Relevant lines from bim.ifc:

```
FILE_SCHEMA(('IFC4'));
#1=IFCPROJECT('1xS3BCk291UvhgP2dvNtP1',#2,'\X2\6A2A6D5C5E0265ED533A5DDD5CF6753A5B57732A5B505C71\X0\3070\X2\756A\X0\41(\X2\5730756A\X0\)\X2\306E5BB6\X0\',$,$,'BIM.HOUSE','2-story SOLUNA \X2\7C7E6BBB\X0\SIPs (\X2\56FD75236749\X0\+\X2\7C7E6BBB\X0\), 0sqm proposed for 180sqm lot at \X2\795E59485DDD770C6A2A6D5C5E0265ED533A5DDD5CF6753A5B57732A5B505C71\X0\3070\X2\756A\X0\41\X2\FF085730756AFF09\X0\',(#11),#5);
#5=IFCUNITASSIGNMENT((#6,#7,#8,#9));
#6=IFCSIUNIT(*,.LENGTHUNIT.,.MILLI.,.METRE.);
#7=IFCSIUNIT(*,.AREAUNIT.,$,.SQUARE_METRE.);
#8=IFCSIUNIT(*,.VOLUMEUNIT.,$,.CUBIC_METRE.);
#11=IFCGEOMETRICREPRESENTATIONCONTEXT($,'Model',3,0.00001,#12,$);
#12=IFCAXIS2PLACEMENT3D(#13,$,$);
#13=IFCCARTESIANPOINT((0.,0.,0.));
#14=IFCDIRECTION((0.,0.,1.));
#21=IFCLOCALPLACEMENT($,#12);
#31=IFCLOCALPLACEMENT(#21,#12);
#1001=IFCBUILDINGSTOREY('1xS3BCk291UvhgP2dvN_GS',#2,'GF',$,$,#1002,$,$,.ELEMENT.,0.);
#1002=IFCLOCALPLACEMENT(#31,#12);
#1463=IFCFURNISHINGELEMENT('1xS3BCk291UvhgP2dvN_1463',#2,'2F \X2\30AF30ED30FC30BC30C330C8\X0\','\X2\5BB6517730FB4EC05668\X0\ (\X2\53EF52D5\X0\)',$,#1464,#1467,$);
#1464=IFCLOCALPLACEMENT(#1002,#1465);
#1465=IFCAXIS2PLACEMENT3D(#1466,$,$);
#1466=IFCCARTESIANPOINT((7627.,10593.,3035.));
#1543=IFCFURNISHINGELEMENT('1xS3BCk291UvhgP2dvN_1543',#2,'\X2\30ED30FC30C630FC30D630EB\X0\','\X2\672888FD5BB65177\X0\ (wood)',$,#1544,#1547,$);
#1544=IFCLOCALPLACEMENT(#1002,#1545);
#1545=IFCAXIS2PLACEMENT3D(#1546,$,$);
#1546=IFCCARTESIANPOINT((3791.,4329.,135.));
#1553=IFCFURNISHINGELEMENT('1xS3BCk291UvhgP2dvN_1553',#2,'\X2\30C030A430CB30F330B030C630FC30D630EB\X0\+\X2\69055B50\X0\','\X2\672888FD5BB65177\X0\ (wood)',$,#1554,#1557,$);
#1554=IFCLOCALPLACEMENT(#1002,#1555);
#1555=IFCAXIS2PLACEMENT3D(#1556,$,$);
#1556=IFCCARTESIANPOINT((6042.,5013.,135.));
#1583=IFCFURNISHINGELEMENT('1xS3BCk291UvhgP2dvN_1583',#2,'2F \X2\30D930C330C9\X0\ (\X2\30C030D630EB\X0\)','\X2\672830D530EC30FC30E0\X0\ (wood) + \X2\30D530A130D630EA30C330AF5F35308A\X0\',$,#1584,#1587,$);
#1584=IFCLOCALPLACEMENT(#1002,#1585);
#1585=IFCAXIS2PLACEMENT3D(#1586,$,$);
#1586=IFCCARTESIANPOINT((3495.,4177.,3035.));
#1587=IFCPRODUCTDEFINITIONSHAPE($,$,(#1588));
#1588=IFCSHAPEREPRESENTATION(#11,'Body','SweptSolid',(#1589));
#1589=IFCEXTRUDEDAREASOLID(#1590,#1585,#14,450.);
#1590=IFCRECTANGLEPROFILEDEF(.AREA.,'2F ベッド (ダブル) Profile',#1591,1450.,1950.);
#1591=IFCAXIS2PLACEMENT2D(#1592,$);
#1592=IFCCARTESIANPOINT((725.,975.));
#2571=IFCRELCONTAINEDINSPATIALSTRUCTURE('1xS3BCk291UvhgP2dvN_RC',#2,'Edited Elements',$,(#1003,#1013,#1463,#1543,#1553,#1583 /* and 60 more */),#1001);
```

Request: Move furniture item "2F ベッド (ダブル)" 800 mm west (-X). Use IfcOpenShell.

```python
import ifcopenshell
import ifcopenshell.api.geometry
import ifcopenshell.util.placement

model = ifcopenshell.open("bim.ifc")

item = model.by_guid("1xS3BCk291UvhgP2dvN_1583")
matrix = ifcopenshell.util.placement.get_local_placement(item.ObjectPlacement)
matrix[0, 3] -= 800.0
ifcopenshell.api.geometry.edit_object_placement(model, product=item, matrix=matrix, is_si=False)

print(ifcopenshell.util.placement.get_local_placement(item.ObjectPlacement).round(3) + 0.0)

model.write("bim_updated.ifc")
```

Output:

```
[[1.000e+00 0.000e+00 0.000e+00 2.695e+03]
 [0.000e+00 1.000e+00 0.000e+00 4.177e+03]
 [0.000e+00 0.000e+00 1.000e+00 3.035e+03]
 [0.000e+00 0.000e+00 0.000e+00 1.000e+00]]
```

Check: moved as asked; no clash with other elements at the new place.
